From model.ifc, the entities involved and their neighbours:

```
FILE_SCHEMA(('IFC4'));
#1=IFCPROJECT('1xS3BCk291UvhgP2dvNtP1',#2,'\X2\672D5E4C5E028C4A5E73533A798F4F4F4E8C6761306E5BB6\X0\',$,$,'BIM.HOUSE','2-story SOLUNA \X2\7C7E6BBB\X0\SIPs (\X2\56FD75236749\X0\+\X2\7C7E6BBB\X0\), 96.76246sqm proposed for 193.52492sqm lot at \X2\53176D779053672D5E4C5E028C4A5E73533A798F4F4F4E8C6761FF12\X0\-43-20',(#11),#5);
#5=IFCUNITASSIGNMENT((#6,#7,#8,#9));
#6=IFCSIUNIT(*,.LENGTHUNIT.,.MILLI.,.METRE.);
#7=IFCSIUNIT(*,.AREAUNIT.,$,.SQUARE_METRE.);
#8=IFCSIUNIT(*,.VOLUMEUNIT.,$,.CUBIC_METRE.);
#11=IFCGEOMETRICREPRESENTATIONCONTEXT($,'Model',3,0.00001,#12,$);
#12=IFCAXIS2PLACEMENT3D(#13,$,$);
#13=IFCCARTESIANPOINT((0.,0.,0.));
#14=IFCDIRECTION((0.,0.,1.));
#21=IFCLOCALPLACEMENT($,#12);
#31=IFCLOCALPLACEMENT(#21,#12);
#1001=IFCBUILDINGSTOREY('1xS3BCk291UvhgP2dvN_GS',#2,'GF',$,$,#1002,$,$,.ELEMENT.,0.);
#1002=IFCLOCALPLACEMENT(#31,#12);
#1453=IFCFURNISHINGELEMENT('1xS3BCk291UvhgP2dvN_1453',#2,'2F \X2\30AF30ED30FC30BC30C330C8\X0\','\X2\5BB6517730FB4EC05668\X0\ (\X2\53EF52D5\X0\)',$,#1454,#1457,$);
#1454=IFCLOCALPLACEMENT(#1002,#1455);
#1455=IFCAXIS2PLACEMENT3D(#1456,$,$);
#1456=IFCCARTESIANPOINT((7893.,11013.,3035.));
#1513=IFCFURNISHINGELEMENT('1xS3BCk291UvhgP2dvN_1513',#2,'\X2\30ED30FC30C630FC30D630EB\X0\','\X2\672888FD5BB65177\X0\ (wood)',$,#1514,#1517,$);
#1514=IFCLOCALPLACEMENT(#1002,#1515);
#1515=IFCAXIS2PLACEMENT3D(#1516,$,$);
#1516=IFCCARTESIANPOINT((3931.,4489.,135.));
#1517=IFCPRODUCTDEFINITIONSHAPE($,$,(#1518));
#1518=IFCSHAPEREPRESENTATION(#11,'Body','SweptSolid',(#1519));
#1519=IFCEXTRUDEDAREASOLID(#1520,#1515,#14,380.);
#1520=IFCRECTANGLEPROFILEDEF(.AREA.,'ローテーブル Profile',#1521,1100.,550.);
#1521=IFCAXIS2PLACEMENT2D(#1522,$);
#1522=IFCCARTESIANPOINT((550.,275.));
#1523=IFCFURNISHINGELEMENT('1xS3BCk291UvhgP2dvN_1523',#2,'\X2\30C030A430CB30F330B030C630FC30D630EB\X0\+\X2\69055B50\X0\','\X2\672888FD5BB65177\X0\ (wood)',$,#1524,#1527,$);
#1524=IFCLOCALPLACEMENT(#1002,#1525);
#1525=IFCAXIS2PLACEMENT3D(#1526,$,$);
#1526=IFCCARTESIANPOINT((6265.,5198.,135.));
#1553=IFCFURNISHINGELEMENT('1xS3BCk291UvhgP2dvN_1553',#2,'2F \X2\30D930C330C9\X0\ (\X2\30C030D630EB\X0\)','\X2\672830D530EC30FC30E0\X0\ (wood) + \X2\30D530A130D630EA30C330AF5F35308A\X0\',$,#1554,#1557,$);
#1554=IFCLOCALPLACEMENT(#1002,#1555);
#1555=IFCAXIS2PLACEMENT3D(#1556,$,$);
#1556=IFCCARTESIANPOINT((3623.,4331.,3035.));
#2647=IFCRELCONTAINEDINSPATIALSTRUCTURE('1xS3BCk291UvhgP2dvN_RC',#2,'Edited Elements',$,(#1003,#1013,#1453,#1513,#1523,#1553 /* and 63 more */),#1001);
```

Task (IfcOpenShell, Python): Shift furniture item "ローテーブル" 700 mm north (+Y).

```python
import ifcopenshell
import ifcopenshell.api.geometry
import ifcopenshell.util.placement

model = ifcopenshell.open("model.ifc")

item = model.by_id(1513)
matrix = ifcopenshell.util.placement.get_local_placement(item.ObjectPlacement)
matrix[1, 3] += 700.0
ifcopenshell.api.geometry.edit_object_placement(model, product=item, matrix=matrix, is_si=False)

print(ifcopenshell.util.placement.get_local_placement(item.ObjectPlacement).round(3) + 0.0)

model.write("model_edited.ifc")
```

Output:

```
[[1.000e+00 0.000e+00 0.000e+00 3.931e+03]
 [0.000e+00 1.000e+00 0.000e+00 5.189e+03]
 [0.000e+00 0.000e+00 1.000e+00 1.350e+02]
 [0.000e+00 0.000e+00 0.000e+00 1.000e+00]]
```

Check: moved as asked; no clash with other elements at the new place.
